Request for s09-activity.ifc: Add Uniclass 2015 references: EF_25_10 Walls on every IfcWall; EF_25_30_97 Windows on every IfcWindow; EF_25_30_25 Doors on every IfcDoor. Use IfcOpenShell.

First a look at what the model holds.

```python
import ifcopenshell

model = ifcopenshell.open("s09-activity.ifc")
print(model.schema)
print("classifications:", [c.Name for c in model.by_type("IfcClassification")])
for ifc_class in ("IfcDoor", "IfcRoof", "IfcStair", "IfcWall", "IfcWindow"):
    print(ifc_class, len(model.by_type(ifc_class)))
```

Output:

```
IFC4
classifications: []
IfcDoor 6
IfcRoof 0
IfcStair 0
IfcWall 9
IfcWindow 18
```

```python
import ifcopenshell
import ifcopenshell.api.classification

model = ifcopenshell.open("s09-activity.ifc")

system = ifcopenshell.api.classification.add_classification(model, classification="Uniclass 2015")

codes = {
    "IfcWall": ("EF_25_10", "Walls"),
    "IfcWindow": ("EF_25_30_97", "Windows"),
    "IfcDoor": ("EF_25_30_25", "Doors"),
}
for ifc_class, (code, name) in codes.items():
    products = model.by_type(ifc_class)
    ifcopenshell.api.classification.add_reference(
        model, products=products, classification=system, identification=code, name=name
    )
    print(code, len(products))

model.write("s09-activity_v2.ifc")
```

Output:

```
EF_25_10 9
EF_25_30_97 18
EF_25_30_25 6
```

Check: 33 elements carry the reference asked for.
